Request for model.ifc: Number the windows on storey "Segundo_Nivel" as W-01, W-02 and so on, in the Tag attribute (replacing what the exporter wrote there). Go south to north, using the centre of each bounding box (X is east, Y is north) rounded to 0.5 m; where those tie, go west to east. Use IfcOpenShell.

First a look at what the model holds.

```python
import ifcopenshell
import ifcopenshell.util.element
import ifcopenshell.util.placement

model = ifcopenshell.open("model.ifc")
print(model.schema)
storey = next(s for s in model.by_type("IfcBuildingStorey") if s.Name == "Segundo_Nivel")
windows = [e for e in ifcopenshell.util.element.get_decomposition(storey) if e.is_a("IfcWindow")]
for e in sorted(windows, key=lambda e: e.id()):
    origin = ifcopenshell.util.placement.get_local_placement(e.ObjectPlacement)[:3, 3]
    print(e.id(), e.Tag, e.Name, origin.round(2) + 0.0, sep=" | ")
```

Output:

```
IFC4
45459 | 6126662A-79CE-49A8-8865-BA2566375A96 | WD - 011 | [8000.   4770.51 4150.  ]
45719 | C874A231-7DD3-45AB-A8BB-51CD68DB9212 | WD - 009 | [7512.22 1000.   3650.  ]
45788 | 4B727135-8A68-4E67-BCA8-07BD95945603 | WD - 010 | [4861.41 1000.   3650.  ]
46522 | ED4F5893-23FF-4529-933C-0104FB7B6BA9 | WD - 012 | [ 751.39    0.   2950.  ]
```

```python
import ifcopenshell
import ifcopenshell.geom
import ifcopenshell.util.element
import ifcopenshell.util.shape

model = ifcopenshell.open("model.ifc")
settings = ifcopenshell.geom.settings()
settings.set("use-world-coords", True)


def centre(element):
    shape = ifcopenshell.geom.create_shape(settings, element)
    return ifcopenshell.util.shape.get_bbox_centroid(shape.geometry)


storey = next(s for s in model.by_type("IfcBuildingStorey") if s.Name == "Segundo_Nivel")
windows = [e for e in ifcopenshell.util.element.get_decomposition(storey) if e.is_a("IfcWindow")]

# Insertion points can sit at a corner or the storey origin, so sort by the geometry (in metres).
centres = {e: centre(e) for e in windows}
windows.sort(key=lambda e: (round(centres[e][1] / 0.5), centres[e][0]))

for i, e in enumerate(windows, start=1):
    number = f"W-{i:02d}"
    e.Tag = number
    print(e.id(), number)

model.write("model-out.ifc")
```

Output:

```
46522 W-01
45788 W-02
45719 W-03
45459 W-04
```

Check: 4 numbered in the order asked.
